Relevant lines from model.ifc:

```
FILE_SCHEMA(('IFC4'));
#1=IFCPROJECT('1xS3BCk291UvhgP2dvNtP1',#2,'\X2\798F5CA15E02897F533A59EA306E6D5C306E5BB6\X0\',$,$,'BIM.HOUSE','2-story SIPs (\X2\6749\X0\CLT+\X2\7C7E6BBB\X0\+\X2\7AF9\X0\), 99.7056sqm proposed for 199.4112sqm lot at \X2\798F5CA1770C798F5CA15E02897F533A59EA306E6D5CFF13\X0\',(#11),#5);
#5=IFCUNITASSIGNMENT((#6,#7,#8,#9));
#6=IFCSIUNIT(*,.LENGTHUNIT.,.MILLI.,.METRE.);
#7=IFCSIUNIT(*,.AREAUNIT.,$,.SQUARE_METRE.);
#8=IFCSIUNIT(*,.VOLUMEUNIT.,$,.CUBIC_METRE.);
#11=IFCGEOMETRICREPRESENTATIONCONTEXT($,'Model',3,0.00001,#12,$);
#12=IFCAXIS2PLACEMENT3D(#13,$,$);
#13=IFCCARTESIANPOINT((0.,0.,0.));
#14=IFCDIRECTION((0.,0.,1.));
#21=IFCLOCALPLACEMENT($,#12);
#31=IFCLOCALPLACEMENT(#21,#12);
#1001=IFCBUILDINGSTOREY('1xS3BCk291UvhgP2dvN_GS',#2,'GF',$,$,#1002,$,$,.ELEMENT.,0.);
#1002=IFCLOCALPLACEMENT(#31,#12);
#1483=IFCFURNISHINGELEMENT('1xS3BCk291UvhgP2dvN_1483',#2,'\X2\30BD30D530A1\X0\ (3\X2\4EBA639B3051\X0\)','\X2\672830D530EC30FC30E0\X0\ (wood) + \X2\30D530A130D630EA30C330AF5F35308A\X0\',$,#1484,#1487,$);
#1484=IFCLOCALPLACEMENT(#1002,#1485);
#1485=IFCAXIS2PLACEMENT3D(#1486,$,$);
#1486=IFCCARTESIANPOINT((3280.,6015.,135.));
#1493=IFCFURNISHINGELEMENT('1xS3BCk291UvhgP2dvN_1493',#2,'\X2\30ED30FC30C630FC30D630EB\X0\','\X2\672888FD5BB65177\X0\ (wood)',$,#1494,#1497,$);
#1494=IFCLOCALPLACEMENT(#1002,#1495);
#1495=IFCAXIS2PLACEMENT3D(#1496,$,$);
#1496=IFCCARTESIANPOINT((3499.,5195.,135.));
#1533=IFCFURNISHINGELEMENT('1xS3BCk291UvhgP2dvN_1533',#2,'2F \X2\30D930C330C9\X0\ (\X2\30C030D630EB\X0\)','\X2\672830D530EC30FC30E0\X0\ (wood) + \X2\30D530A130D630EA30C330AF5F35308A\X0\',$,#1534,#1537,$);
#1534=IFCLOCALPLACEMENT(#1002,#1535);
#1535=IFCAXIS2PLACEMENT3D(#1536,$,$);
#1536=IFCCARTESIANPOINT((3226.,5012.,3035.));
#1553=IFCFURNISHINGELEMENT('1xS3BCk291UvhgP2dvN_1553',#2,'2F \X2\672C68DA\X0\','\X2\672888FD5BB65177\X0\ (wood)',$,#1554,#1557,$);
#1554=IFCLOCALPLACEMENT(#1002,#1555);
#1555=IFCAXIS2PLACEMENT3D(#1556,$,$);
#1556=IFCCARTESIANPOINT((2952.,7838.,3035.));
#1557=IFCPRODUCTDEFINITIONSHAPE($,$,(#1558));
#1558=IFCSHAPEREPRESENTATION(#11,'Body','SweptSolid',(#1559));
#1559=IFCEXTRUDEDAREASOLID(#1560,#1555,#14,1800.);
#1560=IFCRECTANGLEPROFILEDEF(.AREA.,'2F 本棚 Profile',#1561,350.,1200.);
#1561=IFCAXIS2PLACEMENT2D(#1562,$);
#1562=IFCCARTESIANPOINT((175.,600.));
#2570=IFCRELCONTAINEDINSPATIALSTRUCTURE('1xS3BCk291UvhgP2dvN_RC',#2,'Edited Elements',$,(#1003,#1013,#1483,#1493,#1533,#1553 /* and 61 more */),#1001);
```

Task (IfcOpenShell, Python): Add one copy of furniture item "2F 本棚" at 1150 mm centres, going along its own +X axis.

```python
import ifcopenshell
import ifcopenshell.api.geometry
import ifcopenshell.api.root
import ifcopenshell.util.element
import ifcopenshell.util.placement
import ifcopenshell.util.unit

model = ifcopenshell.open("model.ifc")
unit_scale = ifcopenshell.util.unit.calculate_unit_scale(model)


def reuse_history(source, copy):
    """copy_class also copies each property set's owner history, people and application; keep the originals."""
    for rel in copy.IsDefinedBy:
        if rel.is_a("IfcRelDefinesByProperties") and (history := rel.RelatingPropertyDefinition.OwnerHistory):
            rel.RelatingPropertyDefinition.OwnerHistory = source.OwnerHistory
            ifcopenshell.util.element.remove_deep2(model, history)


source = model.by_guid("1xS3BCk291UvhgP2dvN_1553")
base = ifcopenshell.util.placement.get_local_placement(source.ObjectPlacement)
step = base[:3, 0] * 1.15 / unit_scale

for i in range(1, 2):
    copy = ifcopenshell.api.root.copy_class(model, product=source)
    copy.Representation = ifcopenshell.util.element.copy_deep(
        model, source.Representation, exclude=["IfcGeometricRepresentationContext", "IfcRepresentationMap"]
    )
    reuse_history(source, copy)
    matrix = base.copy()
    matrix[:3, 3] += i * step
    print("added at", matrix[:3, 3].round(3) + 0.0)
    ifcopenshell.api.geometry.edit_object_placement(model, product=copy, matrix=matrix, is_si=False)

model.write("model_updated.ifc")
```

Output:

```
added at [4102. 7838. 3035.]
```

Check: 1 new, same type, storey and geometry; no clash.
